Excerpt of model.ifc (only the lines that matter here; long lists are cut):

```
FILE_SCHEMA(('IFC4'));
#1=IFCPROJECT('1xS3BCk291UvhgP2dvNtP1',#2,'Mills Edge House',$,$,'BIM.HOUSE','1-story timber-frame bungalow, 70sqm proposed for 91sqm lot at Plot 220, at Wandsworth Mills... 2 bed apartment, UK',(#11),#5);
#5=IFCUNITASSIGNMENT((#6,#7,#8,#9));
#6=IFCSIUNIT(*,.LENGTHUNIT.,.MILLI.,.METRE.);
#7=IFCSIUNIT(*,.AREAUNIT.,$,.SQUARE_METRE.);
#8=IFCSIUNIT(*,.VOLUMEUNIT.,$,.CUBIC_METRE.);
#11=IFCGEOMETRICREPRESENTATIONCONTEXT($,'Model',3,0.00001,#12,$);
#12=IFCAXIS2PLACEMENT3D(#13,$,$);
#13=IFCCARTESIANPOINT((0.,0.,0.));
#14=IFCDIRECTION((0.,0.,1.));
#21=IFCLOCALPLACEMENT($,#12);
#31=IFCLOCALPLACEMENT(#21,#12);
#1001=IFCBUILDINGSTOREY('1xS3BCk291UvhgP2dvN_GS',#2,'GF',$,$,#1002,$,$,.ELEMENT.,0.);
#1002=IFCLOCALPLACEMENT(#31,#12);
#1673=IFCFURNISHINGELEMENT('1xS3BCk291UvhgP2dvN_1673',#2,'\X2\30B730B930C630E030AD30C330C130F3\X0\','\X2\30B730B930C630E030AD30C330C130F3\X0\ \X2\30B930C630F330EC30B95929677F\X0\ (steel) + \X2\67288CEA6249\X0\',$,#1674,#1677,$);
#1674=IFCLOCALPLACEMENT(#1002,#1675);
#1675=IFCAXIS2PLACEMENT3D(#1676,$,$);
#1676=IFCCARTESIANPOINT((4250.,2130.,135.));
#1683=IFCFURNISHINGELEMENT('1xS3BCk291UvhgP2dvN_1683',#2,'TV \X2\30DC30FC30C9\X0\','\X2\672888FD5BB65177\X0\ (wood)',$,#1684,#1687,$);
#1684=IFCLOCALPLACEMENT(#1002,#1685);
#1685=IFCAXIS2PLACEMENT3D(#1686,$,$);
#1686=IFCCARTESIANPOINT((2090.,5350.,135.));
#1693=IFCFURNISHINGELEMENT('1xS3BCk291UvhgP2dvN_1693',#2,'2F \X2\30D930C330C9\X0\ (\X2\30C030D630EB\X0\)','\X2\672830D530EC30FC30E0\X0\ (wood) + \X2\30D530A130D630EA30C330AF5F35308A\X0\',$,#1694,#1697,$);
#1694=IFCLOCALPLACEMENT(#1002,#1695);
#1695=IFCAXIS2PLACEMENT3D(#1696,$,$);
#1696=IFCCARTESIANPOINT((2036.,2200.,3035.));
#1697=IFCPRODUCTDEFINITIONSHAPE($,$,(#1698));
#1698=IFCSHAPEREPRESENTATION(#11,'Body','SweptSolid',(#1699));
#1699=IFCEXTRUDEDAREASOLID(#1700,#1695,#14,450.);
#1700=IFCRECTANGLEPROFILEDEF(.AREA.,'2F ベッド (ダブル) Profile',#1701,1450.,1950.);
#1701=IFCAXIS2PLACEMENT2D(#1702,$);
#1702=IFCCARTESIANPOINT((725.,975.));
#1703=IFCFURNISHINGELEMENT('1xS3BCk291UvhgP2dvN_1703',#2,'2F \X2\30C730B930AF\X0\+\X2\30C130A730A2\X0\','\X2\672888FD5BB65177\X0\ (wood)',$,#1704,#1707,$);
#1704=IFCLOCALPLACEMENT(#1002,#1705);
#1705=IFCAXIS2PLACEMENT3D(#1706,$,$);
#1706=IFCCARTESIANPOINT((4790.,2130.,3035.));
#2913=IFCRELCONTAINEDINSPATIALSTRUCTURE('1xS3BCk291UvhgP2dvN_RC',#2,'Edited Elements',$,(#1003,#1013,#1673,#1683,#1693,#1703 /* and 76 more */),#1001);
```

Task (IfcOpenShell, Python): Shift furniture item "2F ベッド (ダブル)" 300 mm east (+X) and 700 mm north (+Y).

```python
import ifcopenshell
import ifcopenshell.api.geometry
import ifcopenshell.util.placement

model = ifcopenshell.open("model.ifc")

item = model.by_id(1693)
matrix = ifcopenshell.util.placement.get_local_placement(item.ObjectPlacement)
matrix[0, 3] += 300.0
matrix[1, 3] += 700.0
ifcopenshell.api.geometry.edit_object_placement(model, product=item, matrix=matrix, is_si=False)

print(ifcopenshell.util.placement.get_local_placement(item.ObjectPlacement).round(3) + 0.0)

model.write("model_rev.ifc")
```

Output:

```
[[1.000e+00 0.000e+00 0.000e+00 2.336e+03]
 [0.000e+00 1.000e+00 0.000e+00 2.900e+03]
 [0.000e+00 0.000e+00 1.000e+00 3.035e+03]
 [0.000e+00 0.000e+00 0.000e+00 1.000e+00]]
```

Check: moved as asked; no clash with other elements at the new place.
